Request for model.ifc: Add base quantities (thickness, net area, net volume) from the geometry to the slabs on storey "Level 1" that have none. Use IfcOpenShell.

First a look at what the model holds.

```python
import ifcopenshell
import ifcopenshell.util.element
import ifcopenshell.util.unit

model = ifcopenshell.open("model.ifc")
print(model.schema)
for unit_type in ("LENGTHUNIT", "AREAUNIT", "VOLUMEUNIT"):
    print(unit_type, ifcopenshell.util.unit.calculate_unit_scale(model, unit_type))
storey = next(s for s in model.by_type("IfcBuildingStorey") if s.Name == "Level 1")
slabs = [e for e in ifcopenshell.util.element.get_decomposition(storey) if e.is_a("IfcSlab")]
for e in sorted(slabs, key=lambda e: e.id()):
    print(e.id(), e.is_a(), e.Name, list(ifcopenshell.util.element.get_psets(e, qtos_only=True)), sep=" | ")
```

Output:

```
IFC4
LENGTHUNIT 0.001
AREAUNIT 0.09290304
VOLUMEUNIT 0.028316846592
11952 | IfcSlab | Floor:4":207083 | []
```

```python
import ifcopenshell
import ifcopenshell.api.pset
import ifcopenshell.geom
import ifcopenshell.util.element
import ifcopenshell.util.shape
import ifcopenshell.util.unit

model = ifcopenshell.open("model.ifc")
unit_scale = ifcopenshell.util.unit.calculate_unit_scale(model)
area_scale = ifcopenshell.util.unit.calculate_unit_scale(model, "AREAUNIT")
volume_scale = ifcopenshell.util.unit.calculate_unit_scale(model, "VOLUMEUNIT")
settings = ifcopenshell.geom.settings()

storey = next(s for s in model.by_type("IfcBuildingStorey") if s.Name == "Level 1")
slabs = [e for e in ifcopenshell.util.element.get_decomposition(storey) if e.is_a("IfcSlab")]

for e in sorted(slabs, key=lambda e: e.id()):
    if ifcopenshell.util.element.get_psets(e, qtos_only=True, should_inherit=False):
        continue
    # Geometry comes back in metres, in the element's own axes.
    shape = ifcopenshell.geom.create_shape(settings, e)
    values = {
        "Width": ifcopenshell.util.shape.get_z(shape.geometry) / unit_scale,
        "NetArea": ifcopenshell.util.shape.get_footprint_area(shape.geometry) / area_scale,
        "NetVolume": ifcopenshell.util.shape.get_volume(shape.geometry) / volume_scale,
    }
    qto = ifcopenshell.api.pset.add_qto(model, product=e, name="Qto_SlabBaseQuantities")
    ifcopenshell.api.pset.edit_qto(model, qto=qto, properties=values)
    print(e.id(), {k: round(v, 3) for k, v in values.items()})

model.write("model_v2.ifc")
```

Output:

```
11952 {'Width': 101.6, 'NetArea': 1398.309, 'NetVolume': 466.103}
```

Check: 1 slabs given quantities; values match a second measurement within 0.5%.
